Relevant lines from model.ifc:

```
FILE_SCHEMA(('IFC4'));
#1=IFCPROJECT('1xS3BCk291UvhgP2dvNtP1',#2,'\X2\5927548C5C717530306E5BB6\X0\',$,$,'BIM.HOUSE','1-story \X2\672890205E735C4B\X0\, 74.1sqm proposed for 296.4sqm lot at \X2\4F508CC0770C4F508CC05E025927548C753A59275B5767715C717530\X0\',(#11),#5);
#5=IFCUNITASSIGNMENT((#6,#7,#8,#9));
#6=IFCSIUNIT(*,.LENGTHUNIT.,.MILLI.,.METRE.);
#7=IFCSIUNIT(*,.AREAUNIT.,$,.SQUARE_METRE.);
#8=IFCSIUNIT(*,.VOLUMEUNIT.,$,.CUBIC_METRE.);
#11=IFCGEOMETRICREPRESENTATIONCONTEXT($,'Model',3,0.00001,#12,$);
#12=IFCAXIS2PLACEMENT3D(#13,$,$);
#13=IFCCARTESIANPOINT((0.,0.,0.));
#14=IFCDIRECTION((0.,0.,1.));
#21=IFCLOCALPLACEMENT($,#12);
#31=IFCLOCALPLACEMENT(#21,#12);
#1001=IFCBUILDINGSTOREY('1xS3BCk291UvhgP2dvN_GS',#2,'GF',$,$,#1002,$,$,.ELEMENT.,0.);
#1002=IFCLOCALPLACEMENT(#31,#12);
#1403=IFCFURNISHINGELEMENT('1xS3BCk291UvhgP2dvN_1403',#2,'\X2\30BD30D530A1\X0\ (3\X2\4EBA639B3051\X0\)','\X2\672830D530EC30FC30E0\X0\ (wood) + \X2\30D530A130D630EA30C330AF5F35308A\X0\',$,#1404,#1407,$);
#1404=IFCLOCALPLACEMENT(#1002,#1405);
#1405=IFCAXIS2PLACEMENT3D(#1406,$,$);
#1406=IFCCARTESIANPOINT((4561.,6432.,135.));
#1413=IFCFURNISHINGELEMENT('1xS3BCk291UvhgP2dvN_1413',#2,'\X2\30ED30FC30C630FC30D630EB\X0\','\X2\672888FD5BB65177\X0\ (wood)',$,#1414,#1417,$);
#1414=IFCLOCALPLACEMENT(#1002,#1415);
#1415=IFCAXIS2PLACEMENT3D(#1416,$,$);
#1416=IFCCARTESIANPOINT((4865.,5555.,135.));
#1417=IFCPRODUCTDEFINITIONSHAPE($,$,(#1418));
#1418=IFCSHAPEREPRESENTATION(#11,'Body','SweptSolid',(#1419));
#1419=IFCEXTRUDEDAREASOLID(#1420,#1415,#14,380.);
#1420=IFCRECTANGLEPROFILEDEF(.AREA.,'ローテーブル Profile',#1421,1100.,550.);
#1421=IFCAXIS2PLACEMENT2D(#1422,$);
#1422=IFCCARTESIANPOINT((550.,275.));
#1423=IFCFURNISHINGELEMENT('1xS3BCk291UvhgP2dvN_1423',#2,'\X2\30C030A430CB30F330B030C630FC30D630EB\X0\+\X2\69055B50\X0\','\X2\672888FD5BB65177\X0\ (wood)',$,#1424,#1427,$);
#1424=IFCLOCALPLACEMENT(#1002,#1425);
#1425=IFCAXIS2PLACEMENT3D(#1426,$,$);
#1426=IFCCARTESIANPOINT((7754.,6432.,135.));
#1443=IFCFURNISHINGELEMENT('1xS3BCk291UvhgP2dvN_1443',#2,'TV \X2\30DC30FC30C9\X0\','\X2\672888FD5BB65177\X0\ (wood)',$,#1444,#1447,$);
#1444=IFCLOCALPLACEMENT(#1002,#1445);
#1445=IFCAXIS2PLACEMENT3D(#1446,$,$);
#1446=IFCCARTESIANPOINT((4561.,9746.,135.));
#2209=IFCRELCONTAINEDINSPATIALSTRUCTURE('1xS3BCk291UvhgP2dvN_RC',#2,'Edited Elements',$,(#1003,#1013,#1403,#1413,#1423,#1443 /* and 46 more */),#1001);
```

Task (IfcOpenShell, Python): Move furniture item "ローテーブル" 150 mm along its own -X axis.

```python
import ifcopenshell
import ifcopenshell.api.geometry
import ifcopenshell.util.placement
import ifcopenshell.util.unit

model = ifcopenshell.open("model.ifc")
unit_scale = ifcopenshell.util.unit.calculate_unit_scale(model)

item = model.by_guid("1xS3BCk291UvhgP2dvN_1413")
matrix = ifcopenshell.util.placement.get_local_placement(item.ObjectPlacement)
matrix[:3, 3] -= matrix[:3, 0] * 0.15 / unit_scale
ifcopenshell.api.geometry.edit_object_placement(model, product=item, matrix=matrix, is_si=False)

print(ifcopenshell.util.placement.get_local_placement(item.ObjectPlacement).round(3) + 0.0)

model.write("model_edited.ifc")
```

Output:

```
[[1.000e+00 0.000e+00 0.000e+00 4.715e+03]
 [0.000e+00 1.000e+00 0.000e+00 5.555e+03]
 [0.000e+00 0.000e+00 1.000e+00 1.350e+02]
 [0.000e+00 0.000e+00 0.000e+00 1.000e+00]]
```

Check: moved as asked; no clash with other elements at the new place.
